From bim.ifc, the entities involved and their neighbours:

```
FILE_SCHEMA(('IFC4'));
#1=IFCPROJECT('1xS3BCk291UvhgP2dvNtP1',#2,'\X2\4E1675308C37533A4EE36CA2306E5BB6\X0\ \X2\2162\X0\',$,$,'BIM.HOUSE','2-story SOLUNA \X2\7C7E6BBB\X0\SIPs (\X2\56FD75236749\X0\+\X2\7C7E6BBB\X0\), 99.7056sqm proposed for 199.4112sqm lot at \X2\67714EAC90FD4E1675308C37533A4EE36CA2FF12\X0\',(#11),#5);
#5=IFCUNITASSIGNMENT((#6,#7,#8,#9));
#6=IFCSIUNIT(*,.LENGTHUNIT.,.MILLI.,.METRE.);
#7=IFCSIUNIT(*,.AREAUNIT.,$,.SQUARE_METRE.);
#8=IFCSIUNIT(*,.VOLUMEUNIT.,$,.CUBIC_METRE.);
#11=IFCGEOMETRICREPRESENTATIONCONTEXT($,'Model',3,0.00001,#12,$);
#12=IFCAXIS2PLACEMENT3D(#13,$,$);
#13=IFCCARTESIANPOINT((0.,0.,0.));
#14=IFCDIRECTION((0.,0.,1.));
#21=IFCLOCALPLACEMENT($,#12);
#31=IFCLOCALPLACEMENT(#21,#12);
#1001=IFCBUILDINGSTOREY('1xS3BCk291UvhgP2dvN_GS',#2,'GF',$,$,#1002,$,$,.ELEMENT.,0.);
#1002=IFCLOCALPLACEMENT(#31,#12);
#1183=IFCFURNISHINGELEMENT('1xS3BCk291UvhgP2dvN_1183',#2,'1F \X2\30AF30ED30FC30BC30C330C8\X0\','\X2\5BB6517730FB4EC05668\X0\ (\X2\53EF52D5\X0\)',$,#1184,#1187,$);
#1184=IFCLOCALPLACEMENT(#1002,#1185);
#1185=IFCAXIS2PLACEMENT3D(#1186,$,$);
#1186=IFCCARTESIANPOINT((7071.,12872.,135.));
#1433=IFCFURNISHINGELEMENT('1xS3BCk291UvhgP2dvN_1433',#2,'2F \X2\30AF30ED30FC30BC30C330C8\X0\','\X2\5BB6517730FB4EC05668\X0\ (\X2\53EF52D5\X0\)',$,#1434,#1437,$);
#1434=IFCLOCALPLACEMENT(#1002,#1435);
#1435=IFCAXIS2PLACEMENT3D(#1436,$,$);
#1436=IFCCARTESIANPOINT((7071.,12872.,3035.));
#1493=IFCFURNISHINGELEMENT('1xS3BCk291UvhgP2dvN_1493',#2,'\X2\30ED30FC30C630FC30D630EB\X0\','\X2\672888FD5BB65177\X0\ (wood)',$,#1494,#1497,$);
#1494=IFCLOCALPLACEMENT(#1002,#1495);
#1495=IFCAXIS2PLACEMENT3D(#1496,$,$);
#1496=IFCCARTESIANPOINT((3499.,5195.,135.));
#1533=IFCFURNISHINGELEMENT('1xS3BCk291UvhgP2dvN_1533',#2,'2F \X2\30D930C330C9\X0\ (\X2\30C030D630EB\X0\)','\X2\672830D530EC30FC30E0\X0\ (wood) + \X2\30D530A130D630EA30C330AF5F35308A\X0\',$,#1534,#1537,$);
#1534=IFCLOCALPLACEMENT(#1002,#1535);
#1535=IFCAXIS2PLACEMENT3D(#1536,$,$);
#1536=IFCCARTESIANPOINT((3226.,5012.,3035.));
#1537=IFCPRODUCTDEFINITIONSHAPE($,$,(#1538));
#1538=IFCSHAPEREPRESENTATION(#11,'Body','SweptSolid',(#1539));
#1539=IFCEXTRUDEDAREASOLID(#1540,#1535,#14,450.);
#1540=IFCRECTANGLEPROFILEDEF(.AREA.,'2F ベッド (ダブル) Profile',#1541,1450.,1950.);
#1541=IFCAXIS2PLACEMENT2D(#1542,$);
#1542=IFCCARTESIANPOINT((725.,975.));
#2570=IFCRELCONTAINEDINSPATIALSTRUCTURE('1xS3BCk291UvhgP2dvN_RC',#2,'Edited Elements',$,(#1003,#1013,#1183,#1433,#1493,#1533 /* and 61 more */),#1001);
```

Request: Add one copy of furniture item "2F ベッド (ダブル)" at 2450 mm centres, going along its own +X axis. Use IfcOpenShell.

```python
import ifcopenshell
import ifcopenshell.api.geometry
import ifcopenshell.api.root
import ifcopenshell.util.element
import ifcopenshell.util.placement
import ifcopenshell.util.unit

model = ifcopenshell.open("bim.ifc")
unit_scale = ifcopenshell.util.unit.calculate_unit_scale(model)


def reuse_history(source, copy):
    """copy_class also copies each property set's owner history, people and application; keep the originals."""
    for rel in copy.IsDefinedBy:
        if rel.is_a("IfcRelDefinesByProperties") and (history := rel.RelatingPropertyDefinition.OwnerHistory):
            rel.RelatingPropertyDefinition.OwnerHistory = source.OwnerHistory
            ifcopenshell.util.element.remove_deep2(model, history)


source = model.by_guid("1xS3BCk291UvhgP2dvN_1533")
base = ifcopenshell.util.placement.get_local_placement(source.ObjectPlacement)
step = base[:3, 0] * 2.45 / unit_scale

for i in range(1, 2):
    copy = ifcopenshell.api.root.copy_class(model, product=source)
    copy.Representation = ifcopenshell.util.element.copy_deep(
        model, source.Representation, exclude=["IfcGeometricRepresentationContext", "IfcRepresentationMap"]
    )
    reuse_history(source, copy)
    matrix = base.copy()
    matrix[:3, 3] += i * step
    print("added at", matrix[:3, 3].round(3) + 0.0)
    ifcopenshell.api.geometry.edit_object_placement(model, product=copy, matrix=matrix, is_si=False)

model.write("bim_edited.ifc")
```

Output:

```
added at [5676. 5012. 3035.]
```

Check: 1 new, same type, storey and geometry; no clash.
